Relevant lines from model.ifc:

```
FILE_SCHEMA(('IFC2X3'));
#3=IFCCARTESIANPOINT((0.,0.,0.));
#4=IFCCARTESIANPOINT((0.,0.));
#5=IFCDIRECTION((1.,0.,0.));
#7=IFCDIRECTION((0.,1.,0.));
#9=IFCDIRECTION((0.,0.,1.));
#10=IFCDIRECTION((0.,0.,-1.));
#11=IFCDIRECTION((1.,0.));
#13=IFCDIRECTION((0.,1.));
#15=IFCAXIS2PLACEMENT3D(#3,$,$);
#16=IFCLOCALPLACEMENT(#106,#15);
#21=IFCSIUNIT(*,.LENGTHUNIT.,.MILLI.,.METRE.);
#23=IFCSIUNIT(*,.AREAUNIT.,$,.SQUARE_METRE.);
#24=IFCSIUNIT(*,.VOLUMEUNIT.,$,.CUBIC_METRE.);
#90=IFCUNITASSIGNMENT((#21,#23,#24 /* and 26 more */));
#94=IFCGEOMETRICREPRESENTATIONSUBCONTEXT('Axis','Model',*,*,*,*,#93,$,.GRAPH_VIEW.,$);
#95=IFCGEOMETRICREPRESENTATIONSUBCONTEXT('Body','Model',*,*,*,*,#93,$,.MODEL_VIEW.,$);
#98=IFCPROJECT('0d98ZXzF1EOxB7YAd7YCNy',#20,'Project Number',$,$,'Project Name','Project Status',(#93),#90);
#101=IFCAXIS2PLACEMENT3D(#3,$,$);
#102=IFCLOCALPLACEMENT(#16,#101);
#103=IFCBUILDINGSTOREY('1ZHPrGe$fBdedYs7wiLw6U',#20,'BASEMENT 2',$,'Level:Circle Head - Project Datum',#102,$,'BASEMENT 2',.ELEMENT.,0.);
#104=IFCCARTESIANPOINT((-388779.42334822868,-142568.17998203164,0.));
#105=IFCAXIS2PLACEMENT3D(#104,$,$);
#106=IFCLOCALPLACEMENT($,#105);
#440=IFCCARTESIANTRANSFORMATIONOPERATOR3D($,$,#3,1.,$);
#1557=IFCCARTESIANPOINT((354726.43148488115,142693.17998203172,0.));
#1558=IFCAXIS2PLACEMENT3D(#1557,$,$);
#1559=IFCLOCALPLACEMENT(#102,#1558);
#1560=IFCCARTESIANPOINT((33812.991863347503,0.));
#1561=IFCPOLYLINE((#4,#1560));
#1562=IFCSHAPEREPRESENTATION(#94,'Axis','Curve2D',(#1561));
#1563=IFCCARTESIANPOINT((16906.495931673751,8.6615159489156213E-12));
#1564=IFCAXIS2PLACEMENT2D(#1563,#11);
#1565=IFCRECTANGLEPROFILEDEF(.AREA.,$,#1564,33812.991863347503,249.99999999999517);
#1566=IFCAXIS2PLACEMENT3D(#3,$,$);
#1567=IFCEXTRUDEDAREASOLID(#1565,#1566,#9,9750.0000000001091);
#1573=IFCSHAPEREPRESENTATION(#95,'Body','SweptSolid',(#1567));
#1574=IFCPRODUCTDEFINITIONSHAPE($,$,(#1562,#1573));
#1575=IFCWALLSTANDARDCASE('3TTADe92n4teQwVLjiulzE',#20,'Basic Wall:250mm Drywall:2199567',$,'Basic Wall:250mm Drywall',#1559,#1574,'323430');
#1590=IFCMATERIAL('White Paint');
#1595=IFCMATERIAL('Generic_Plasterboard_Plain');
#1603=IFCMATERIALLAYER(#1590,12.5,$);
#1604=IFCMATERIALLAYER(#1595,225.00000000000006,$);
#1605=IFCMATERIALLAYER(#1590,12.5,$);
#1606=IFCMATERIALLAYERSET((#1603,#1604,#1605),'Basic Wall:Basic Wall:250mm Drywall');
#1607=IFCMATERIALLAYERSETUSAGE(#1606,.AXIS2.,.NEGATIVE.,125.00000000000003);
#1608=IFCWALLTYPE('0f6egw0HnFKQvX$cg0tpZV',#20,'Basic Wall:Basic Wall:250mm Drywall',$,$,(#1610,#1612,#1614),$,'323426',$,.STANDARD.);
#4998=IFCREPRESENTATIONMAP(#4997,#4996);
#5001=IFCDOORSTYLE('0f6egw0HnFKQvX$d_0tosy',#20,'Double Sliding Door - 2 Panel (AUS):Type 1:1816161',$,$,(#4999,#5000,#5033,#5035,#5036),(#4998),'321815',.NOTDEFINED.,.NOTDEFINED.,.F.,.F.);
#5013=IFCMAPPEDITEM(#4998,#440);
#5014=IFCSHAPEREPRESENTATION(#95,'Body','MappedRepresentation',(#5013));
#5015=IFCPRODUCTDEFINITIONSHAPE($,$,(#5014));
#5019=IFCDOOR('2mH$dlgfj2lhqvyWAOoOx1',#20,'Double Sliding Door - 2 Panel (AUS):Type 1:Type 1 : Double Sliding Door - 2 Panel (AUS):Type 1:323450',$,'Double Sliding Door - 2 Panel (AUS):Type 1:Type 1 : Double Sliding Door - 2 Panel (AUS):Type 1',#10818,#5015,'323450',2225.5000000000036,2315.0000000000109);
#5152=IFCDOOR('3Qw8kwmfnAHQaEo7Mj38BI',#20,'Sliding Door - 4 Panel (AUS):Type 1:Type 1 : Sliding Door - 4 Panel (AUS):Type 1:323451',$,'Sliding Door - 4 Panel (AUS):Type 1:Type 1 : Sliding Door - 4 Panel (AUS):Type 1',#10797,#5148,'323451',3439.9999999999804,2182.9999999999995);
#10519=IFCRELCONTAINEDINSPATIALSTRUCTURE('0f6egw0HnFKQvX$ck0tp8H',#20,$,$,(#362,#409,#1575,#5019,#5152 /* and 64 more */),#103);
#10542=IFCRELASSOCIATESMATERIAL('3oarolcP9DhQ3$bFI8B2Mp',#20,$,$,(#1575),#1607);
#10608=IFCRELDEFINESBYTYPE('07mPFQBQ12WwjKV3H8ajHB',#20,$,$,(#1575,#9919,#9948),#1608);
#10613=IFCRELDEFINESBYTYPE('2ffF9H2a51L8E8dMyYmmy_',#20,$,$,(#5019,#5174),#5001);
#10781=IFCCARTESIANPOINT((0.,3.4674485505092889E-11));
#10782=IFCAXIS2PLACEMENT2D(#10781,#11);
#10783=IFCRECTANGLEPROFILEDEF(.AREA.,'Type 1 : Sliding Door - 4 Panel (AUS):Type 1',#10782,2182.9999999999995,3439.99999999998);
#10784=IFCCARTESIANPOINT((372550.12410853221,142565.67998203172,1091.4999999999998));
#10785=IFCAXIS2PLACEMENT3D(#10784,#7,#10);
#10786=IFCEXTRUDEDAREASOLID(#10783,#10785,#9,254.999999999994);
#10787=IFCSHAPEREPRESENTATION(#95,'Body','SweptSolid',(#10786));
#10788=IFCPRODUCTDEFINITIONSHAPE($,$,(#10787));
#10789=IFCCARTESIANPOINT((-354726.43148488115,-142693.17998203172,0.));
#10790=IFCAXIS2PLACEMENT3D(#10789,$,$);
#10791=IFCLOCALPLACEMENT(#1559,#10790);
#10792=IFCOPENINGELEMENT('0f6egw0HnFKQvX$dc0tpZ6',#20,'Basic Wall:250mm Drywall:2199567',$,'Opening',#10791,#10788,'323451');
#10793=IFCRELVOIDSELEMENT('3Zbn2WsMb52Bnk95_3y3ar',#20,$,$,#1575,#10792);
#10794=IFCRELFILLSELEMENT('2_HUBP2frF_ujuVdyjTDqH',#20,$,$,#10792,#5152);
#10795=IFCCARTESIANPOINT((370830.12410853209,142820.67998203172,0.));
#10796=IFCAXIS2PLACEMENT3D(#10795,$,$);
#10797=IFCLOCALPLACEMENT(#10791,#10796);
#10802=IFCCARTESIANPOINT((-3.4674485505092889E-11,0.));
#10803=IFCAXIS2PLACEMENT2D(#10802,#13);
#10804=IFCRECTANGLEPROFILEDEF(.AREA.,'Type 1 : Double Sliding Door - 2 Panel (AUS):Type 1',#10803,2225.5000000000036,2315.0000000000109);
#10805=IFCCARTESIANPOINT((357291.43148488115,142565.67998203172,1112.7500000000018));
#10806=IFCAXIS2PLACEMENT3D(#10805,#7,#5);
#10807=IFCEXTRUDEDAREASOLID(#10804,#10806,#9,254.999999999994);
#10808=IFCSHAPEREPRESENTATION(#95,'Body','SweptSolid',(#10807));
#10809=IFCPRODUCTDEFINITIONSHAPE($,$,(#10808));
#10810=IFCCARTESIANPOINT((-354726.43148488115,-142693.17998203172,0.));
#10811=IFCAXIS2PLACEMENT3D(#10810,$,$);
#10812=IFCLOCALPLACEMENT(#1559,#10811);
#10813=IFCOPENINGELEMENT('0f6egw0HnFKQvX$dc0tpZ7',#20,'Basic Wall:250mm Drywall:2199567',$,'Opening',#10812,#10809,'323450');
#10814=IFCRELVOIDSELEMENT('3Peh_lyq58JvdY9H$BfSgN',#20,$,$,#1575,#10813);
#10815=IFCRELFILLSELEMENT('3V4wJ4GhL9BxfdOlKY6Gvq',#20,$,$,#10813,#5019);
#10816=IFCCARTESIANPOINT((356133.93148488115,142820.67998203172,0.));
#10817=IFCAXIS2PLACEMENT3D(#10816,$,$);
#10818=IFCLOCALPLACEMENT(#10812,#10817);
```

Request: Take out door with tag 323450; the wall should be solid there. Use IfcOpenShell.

```python
import ifcopenshell
import ifcopenshell.api.feature
import ifcopenshell.api.root
import ifcopenshell.geom
import ifcopenshell.util.shape

model = ifcopenshell.open("model.ifc")
settings = ifcopenshell.geom.settings()


def volume(element):
    """Net volume in cubic metres, openings subtracted."""
    shape = ifcopenshell.geom.create_shape(settings, element)
    return ifcopenshell.util.shape.get_volume(shape.geometry)


door = model.by_guid("2mH$dlgfj2lhqvyWAOoOx1")
opening = door.FillsVoids[0].RelatingOpeningElement
wall = opening.VoidsElements[0].RelatingBuildingElement
before = volume(wall)

ifcopenshell.api.root.remove_product(model, product=door)
ifcopenshell.api.feature.remove_feature(model, feature=opening)

after = volume(wall)

print(f"wall volume {before:.3f} -> {after:.3f} m3")

model.write("model_rev.ifc")
```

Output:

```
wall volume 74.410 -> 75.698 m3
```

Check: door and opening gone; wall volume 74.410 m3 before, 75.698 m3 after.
